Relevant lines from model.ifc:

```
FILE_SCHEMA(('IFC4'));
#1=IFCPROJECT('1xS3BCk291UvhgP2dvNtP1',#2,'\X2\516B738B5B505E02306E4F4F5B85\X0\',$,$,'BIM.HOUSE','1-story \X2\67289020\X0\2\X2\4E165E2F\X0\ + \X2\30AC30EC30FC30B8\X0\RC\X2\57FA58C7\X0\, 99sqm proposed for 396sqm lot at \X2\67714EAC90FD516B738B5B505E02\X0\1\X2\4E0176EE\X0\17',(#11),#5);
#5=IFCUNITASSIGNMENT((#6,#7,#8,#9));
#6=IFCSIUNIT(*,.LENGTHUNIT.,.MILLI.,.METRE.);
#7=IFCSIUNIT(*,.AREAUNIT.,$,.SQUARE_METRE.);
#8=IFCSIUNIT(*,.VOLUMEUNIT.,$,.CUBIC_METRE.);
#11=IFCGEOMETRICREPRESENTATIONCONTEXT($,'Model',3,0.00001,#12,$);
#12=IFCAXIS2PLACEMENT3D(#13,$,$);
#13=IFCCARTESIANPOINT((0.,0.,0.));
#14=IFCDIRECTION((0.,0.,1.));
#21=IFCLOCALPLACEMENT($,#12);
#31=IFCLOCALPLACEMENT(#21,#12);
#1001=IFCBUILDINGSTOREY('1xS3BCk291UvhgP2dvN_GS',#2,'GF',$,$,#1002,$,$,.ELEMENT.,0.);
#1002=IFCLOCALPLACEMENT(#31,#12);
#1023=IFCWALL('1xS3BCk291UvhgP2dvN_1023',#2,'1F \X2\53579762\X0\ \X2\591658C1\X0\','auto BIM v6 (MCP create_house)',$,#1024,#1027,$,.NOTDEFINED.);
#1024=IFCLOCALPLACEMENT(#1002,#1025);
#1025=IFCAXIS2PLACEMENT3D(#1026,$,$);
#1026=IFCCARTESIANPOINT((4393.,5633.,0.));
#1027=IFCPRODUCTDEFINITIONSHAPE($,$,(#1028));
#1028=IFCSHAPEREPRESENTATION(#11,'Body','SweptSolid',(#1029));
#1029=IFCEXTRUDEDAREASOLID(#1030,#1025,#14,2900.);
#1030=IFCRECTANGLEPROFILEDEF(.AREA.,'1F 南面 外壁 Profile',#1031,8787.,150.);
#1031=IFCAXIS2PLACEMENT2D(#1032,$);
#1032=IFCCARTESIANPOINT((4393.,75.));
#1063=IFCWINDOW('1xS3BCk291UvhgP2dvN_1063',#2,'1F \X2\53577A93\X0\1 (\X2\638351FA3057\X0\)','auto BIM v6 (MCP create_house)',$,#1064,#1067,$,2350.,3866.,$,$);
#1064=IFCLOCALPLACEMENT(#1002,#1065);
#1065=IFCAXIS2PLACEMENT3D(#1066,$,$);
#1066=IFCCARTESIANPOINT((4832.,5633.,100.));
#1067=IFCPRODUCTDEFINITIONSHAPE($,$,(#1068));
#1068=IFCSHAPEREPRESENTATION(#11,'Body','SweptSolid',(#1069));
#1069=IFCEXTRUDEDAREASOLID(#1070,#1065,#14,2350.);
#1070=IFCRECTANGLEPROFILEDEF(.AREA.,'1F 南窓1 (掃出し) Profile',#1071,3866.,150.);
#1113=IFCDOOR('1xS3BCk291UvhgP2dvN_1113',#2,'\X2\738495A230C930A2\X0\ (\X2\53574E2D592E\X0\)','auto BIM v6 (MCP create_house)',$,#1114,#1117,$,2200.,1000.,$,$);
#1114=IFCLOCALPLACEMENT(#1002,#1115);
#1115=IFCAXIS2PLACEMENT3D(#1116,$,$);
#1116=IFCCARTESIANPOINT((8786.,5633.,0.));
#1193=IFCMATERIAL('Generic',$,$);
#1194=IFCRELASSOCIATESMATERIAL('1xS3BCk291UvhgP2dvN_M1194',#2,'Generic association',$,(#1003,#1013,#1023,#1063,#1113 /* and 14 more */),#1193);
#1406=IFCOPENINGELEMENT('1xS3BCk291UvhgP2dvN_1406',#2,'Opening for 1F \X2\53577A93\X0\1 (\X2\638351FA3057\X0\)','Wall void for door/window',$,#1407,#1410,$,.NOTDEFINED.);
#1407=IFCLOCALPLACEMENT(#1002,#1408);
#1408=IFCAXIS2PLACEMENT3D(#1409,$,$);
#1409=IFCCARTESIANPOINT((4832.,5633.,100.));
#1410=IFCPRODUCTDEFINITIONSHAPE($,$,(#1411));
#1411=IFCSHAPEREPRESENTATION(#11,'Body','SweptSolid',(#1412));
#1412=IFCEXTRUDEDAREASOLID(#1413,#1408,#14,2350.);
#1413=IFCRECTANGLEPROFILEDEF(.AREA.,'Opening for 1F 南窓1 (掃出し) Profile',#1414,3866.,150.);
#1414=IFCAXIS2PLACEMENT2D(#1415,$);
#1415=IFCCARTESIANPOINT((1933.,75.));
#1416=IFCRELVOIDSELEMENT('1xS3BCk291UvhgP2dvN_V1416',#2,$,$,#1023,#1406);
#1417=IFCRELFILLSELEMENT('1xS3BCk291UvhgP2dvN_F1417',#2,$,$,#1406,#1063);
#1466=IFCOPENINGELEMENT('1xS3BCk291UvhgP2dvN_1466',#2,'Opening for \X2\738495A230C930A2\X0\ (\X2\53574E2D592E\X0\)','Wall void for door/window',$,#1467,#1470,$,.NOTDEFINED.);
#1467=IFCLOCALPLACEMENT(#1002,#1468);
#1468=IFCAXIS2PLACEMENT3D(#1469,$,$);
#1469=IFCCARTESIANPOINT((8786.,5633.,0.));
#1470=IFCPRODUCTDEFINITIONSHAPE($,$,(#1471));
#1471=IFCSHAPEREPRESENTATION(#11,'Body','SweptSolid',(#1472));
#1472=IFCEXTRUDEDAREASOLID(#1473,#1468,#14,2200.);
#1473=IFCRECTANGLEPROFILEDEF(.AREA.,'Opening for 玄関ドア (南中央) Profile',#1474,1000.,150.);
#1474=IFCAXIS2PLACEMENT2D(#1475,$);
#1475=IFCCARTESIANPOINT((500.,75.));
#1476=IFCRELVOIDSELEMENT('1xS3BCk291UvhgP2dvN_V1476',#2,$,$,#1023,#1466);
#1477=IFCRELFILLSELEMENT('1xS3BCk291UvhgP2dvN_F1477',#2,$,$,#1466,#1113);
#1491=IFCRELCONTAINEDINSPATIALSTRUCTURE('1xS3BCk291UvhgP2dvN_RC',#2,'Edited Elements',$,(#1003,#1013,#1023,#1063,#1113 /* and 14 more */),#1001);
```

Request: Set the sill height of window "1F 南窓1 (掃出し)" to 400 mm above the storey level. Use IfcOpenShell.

```python
import numpy as np
import ifcopenshell
import ifcopenshell.api.geometry
import ifcopenshell.geom
import ifcopenshell.util.element
import ifcopenshell.util.placement
import ifcopenshell.util.shape
import ifcopenshell.util.unit

model = ifcopenshell.open("model.ifc")
unit_scale = ifcopenshell.util.unit.calculate_unit_scale(model)

window = model.by_guid("1xS3BCk291UvhgP2dvN_1063")
opening = window.FillsVoids[0].RelatingOpeningElement
storey = ifcopenshell.util.element.get_container(window, ifc_class="IfcBuildingStorey")
level = ifcopenshell.util.placement.get_local_placement(storey.ObjectPlacement)[2, 3]

# The opening's origin need not be at the sill, so measure its lowest point.
shape = ifcopenshell.geom.create_shape(ifcopenshell.geom.settings(), opening)
bottom = ifcopenshell.util.shape.get_shape_bottom_elevation(shape, shape.geometry) / unit_scale
dz = level + 400.0 - bottom

shift = np.array([0.0, 0.0, dz])
# The window is not placed relative to its opening, so move both.
for product in (opening, window):
    matrix = ifcopenshell.util.placement.get_local_placement(product.ObjectPlacement)
    matrix[:3, 3] += shift
    ifcopenshell.api.geometry.edit_object_placement(model, product=product, matrix=matrix, is_si=False)

print(f"moved by {dz * unit_scale:+.3f} m")

model.write("model_v2.ifc")
```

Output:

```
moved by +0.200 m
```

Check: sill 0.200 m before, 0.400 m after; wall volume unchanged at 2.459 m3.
